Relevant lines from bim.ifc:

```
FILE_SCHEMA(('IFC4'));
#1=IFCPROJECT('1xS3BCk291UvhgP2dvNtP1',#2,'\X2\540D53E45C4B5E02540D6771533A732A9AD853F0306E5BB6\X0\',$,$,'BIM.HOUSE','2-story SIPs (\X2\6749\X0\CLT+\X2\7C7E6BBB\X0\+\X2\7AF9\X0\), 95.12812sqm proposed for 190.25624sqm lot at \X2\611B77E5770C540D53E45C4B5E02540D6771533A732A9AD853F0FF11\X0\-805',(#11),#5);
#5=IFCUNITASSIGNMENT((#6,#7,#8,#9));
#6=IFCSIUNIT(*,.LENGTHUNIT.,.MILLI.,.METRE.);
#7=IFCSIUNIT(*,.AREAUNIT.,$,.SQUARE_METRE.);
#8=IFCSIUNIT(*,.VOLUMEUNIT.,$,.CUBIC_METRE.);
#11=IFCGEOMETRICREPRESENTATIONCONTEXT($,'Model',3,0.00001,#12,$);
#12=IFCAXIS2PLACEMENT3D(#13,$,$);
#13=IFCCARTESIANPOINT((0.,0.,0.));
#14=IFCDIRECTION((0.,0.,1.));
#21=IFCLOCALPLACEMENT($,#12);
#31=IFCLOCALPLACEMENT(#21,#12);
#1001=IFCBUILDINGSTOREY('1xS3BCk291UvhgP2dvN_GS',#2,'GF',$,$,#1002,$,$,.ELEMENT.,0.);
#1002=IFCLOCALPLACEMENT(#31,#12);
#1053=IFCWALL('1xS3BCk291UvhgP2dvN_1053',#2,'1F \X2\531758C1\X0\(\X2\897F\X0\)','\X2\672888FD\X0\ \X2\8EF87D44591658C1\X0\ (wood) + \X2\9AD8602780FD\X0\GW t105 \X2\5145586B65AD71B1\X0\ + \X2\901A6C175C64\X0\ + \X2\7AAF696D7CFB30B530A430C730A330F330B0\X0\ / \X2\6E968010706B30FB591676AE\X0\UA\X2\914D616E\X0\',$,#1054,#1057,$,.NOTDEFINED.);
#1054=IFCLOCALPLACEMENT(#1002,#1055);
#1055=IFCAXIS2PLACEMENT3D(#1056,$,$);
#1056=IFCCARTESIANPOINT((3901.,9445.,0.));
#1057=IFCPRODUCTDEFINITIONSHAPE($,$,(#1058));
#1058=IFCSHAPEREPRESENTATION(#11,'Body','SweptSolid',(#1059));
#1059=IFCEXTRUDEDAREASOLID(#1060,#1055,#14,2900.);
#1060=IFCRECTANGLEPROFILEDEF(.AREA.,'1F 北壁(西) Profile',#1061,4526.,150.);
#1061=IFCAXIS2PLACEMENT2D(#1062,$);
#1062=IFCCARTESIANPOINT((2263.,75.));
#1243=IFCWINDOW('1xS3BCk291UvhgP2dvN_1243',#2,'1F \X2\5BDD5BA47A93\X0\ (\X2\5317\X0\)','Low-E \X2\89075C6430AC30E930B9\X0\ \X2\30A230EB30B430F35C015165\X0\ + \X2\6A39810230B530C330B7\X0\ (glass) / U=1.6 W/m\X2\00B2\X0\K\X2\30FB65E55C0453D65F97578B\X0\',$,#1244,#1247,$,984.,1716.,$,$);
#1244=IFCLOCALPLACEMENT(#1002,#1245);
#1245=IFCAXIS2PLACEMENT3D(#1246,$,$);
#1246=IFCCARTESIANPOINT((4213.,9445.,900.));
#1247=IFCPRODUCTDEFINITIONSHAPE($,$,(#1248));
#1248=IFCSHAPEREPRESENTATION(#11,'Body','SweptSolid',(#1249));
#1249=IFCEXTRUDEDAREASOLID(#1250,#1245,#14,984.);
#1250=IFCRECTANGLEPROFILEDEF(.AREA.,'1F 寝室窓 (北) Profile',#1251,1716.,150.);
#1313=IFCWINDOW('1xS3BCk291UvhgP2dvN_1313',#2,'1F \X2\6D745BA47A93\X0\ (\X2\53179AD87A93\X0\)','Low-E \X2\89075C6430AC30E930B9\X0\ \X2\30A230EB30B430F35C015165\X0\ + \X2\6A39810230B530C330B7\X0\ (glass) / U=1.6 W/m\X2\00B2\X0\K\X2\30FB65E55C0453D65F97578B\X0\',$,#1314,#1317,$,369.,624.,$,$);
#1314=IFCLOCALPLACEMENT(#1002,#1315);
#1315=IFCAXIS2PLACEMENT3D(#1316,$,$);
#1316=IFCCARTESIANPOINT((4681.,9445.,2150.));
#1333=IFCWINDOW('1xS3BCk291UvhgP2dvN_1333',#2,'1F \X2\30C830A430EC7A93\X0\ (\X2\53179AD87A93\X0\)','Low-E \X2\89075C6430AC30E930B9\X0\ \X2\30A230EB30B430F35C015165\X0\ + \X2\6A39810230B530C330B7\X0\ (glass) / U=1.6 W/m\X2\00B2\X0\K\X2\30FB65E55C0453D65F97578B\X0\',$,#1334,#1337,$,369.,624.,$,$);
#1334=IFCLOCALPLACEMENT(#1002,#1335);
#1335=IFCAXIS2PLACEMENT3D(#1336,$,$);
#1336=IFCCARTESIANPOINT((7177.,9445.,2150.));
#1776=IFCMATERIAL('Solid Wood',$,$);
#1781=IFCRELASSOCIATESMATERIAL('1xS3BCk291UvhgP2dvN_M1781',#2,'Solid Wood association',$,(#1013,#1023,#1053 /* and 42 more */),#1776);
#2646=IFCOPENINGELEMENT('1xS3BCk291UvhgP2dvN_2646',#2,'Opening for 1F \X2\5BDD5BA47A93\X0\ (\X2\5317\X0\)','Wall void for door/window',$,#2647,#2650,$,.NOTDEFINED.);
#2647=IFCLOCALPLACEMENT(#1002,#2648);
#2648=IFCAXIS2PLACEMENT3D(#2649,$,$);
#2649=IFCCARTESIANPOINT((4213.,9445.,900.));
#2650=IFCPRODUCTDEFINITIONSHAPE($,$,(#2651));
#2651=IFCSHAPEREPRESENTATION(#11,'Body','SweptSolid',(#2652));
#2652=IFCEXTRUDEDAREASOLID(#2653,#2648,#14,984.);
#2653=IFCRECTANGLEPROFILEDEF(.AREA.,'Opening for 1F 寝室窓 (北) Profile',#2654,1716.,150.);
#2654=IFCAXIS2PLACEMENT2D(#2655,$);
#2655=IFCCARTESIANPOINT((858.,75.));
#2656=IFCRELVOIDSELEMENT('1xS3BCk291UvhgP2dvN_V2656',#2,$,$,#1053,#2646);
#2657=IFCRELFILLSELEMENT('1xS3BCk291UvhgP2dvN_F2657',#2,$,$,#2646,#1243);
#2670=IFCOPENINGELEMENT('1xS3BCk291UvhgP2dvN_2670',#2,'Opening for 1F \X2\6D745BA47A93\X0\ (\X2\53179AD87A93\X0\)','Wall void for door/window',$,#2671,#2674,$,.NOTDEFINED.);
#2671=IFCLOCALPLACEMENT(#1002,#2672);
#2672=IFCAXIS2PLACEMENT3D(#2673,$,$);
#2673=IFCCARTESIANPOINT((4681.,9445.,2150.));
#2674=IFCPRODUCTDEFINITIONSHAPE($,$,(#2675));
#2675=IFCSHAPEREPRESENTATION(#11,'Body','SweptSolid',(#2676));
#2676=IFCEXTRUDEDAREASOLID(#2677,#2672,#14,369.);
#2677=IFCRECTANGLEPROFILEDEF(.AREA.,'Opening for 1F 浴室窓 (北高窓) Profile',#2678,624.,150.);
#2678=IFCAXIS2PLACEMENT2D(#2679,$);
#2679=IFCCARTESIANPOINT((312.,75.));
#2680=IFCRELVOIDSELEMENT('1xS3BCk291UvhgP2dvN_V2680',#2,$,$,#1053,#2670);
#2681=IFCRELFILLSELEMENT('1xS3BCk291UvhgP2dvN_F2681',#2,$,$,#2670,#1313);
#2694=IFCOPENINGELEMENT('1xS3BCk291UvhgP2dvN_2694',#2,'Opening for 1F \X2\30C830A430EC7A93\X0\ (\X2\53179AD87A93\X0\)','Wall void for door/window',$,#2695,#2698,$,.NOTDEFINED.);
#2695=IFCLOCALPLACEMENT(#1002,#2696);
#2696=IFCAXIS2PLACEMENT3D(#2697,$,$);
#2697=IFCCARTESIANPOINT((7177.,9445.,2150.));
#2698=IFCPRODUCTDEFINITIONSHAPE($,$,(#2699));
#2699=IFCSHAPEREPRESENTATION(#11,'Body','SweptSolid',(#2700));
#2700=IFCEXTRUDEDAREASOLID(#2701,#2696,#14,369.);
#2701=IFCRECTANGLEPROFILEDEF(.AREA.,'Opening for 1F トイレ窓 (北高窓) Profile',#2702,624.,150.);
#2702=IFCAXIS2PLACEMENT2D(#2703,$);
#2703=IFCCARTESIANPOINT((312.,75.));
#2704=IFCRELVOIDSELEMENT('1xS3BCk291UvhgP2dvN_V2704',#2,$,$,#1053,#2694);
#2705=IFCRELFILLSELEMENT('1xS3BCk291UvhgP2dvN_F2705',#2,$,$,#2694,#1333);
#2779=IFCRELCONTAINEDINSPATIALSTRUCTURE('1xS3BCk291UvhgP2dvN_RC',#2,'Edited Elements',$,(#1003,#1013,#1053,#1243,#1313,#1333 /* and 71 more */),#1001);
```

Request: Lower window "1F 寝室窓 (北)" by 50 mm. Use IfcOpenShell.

```python
import numpy as np
import ifcopenshell
import ifcopenshell.api.geometry
import ifcopenshell.util.placement
import ifcopenshell.util.unit

model = ifcopenshell.open("bim.ifc")
unit_scale = ifcopenshell.util.unit.calculate_unit_scale(model)

window = model.by_guid("1xS3BCk291UvhgP2dvN_1243")
opening = window.FillsVoids[0].RelatingOpeningElement
dz = -0.05 / unit_scale

shift = np.array([0.0, 0.0, dz])
# The window is not placed relative to its opening, so move both.
for product in (opening, window):
    matrix = ifcopenshell.util.placement.get_local_placement(product.ObjectPlacement)
    matrix[:3, 3] += shift
    ifcopenshell.api.geometry.edit_object_placement(model, product=product, matrix=matrix, is_si=False)

print(f"moved by {dz * unit_scale:+.3f} m")

model.write("bim_v2.ifc")
```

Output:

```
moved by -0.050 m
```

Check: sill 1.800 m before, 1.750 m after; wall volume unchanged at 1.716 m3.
